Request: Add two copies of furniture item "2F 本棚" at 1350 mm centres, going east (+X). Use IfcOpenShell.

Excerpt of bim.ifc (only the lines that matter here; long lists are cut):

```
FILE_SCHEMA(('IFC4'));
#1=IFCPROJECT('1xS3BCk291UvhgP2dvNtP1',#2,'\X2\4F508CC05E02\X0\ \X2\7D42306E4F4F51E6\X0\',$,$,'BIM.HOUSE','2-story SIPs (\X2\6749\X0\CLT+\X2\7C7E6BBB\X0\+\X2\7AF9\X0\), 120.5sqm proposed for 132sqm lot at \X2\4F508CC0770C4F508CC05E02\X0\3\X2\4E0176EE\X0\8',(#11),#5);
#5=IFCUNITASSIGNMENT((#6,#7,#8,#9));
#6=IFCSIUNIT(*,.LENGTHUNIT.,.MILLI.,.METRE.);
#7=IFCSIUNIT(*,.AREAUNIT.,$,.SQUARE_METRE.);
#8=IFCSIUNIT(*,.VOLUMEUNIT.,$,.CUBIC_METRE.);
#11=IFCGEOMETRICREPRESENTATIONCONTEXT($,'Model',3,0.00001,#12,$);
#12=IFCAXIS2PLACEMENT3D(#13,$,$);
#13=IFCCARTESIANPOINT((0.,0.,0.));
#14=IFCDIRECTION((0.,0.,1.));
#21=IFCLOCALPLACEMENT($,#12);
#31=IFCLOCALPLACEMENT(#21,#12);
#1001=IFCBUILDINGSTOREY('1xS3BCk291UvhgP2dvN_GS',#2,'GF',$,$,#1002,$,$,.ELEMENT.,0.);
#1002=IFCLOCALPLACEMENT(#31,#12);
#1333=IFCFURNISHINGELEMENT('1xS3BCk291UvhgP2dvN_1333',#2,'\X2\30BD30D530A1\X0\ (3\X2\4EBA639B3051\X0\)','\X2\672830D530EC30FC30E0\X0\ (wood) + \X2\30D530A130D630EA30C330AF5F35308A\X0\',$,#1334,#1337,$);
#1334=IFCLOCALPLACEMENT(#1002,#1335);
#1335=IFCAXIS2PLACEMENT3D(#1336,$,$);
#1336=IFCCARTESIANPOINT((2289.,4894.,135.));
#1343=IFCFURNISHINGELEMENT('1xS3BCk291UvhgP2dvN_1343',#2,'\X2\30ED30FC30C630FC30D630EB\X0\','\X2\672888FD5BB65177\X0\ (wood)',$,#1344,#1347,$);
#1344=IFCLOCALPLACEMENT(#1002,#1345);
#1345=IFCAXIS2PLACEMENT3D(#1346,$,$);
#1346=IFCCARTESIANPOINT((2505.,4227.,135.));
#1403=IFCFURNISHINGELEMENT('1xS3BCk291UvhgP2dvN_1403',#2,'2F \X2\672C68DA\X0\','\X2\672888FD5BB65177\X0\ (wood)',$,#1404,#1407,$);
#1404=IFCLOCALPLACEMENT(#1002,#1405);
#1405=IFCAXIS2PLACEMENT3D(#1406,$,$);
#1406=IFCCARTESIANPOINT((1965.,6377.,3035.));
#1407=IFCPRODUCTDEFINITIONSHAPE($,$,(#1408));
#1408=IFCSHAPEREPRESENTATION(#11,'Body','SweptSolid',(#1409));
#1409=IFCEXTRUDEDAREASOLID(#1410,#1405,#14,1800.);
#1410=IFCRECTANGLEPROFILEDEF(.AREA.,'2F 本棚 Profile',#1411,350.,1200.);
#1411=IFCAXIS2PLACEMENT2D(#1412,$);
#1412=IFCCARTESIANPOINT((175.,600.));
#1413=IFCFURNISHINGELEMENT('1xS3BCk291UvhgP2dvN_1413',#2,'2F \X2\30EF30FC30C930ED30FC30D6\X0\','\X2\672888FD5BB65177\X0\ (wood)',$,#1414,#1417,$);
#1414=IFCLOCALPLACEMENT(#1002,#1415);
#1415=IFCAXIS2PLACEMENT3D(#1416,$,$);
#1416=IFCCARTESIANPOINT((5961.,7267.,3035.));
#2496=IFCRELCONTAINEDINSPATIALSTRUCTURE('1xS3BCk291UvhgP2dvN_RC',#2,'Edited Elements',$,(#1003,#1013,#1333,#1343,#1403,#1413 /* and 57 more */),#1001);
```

```python
import numpy as np
import ifcopenshell
import ifcopenshell.api.geometry
import ifcopenshell.api.root
import ifcopenshell.util.element
import ifcopenshell.util.placement
import ifcopenshell.util.unit

model = ifcopenshell.open("bim.ifc")
unit_scale = ifcopenshell.util.unit.calculate_unit_scale(model)


def reuse_history(source, copy):
    """copy_class also copies each property set's owner history, people and application; keep the originals."""
    for rel in copy.IsDefinedBy:
        if rel.is_a("IfcRelDefinesByProperties") and (history := rel.RelatingPropertyDefinition.OwnerHistory):
            rel.RelatingPropertyDefinition.OwnerHistory = source.OwnerHistory
            ifcopenshell.util.element.remove_deep2(model, history)


source = model.by_guid("1xS3BCk291UvhgP2dvN_1403")
base = ifcopenshell.util.placement.get_local_placement(source.ObjectPlacement)
step = np.array([1.0, 0.0, 0.0]) * 1.35 / unit_scale

for i in range(1, 3):
    copy = ifcopenshell.api.root.copy_class(model, product=source)
    copy.Representation = ifcopenshell.util.element.copy_deep(
        model, source.Representation, exclude=["IfcGeometricRepresentationContext", "IfcRepresentationMap"]
    )
    reuse_history(source, copy)
    matrix = base.copy()
    matrix[:3, 3] += i * step
    print("added at", matrix[:3, 3].round(3) + 0.0)
    ifcopenshell.api.geometry.edit_object_placement(model, product=copy, matrix=matrix, is_si=False)

model.write("bim_rev.ifc")
```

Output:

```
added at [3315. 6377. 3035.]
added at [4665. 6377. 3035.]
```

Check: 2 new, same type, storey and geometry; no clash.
